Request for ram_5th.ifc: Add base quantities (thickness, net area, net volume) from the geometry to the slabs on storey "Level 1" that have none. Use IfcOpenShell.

First a look at what the model holds.

```python
import ifcopenshell
import ifcopenshell.util.element
import ifcopenshell.util.unit

model = ifcopenshell.open("ram_5th.ifc")
print(model.schema)
for unit_type in ("LENGTHUNIT", "AREAUNIT", "VOLUMEUNIT"):
    print(unit_type, ifcopenshell.util.unit.calculate_unit_scale(model, unit_type))
storey = next(s for s in model.by_type("IfcBuildingStorey") if s.Name == "Level 1")
slabs = [e for e in ifcopenshell.util.element.get_decomposition(storey) if e.is_a("IfcSlab")]
for e in sorted(slabs, key=lambda e: e.id()):
    print(e.id(), e.is_a(), e.Name, list(ifcopenshell.util.element.get_psets(e, qtos_only=True)), sep=" | ")
```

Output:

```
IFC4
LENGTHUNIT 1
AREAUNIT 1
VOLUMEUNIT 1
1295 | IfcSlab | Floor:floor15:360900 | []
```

```python
import ifcopenshell
import ifcopenshell.api.pset
import ifcopenshell.geom
import ifcopenshell.util.element
import ifcopenshell.util.shape
import ifcopenshell.util.unit

model = ifcopenshell.open("ram_5th.ifc")
unit_scale = ifcopenshell.util.unit.calculate_unit_scale(model)
area_scale = ifcopenshell.util.unit.calculate_unit_scale(model, "AREAUNIT")
volume_scale = ifcopenshell.util.unit.calculate_unit_scale(model, "VOLUMEUNIT")
settings = ifcopenshell.geom.settings()

storey = next(s for s in model.by_type("IfcBuildingStorey") if s.Name == "Level 1")
slabs = [e for e in ifcopenshell.util.element.get_decomposition(storey) if e.is_a("IfcSlab")]

for e in sorted(slabs, key=lambda e: e.id()):
    if ifcopenshell.util.element.get_psets(e, qtos_only=True, should_inherit=False):
        continue
    # Geometry comes back in metres, in the element's own axes.
    shape = ifcopenshell.geom.create_shape(settings, e)
    values = {
        "Width": ifcopenshell.util.shape.get_z(shape.geometry) / unit_scale,
        "NetArea": ifcopenshell.util.shape.get_footprint_area(shape.geometry) / area_scale,
        "NetVolume": ifcopenshell.util.shape.get_volume(shape.geometry) / volume_scale,
    }
    qto = ifcopenshell.api.pset.add_qto(model, product=e, name="Qto_SlabBaseQuantities")
    ifcopenshell.api.pset.edit_qto(model, qto=qto, properties=values)
    print(e.id(), {k: round(v, 3) for k, v in values.items()})

model.write("ram_5th_v2.ifc")
```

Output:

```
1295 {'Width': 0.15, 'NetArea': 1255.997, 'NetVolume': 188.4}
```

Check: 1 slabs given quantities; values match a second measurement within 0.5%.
